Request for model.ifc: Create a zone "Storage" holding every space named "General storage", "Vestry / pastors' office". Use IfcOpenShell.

First a look at what the model holds.

```python
import ifcopenshell

model = ifcopenshell.open("model.ifc")
print(model.schema)
seen = {}
for space in model.by_type("IfcSpace"):
    seen[space.LongName] = seen.get(space.LongName, 0) + 1
for name, count in sorted(seen.items(), key=str):
    print(count, "x", name)
print("zones:", [z.Name for z in model.by_type("IfcZone")][:20])
```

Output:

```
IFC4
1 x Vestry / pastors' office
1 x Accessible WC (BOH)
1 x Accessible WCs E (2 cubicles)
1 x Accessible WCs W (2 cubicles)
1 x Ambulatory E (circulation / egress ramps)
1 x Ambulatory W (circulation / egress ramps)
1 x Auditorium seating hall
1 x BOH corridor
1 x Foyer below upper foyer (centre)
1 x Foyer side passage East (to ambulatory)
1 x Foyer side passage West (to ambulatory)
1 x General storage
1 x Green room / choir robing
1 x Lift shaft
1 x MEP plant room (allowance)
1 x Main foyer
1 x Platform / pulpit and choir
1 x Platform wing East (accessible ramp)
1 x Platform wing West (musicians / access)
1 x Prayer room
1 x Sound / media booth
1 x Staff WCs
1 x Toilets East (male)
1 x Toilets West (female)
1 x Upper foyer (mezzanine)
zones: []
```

```python
import ifcopenshell
import ifcopenshell.api.group
import ifcopenshell.api.root

model = ifcopenshell.open("model.ifc")

names = {"General storage", "Vestry / pastors' office"}
spaces = [s for s in model.by_type("IfcSpace") if s.LongName in names]

zone = ifcopenshell.api.root.create_entity(model, ifc_class="IfcZone", name="Storage")
ifcopenshell.api.group.assign_group(model, products=spaces, group=zone)
print(len(spaces), "spaces in", zone.Name)

model.write("model-out.ifc")
```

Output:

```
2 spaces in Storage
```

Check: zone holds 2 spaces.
